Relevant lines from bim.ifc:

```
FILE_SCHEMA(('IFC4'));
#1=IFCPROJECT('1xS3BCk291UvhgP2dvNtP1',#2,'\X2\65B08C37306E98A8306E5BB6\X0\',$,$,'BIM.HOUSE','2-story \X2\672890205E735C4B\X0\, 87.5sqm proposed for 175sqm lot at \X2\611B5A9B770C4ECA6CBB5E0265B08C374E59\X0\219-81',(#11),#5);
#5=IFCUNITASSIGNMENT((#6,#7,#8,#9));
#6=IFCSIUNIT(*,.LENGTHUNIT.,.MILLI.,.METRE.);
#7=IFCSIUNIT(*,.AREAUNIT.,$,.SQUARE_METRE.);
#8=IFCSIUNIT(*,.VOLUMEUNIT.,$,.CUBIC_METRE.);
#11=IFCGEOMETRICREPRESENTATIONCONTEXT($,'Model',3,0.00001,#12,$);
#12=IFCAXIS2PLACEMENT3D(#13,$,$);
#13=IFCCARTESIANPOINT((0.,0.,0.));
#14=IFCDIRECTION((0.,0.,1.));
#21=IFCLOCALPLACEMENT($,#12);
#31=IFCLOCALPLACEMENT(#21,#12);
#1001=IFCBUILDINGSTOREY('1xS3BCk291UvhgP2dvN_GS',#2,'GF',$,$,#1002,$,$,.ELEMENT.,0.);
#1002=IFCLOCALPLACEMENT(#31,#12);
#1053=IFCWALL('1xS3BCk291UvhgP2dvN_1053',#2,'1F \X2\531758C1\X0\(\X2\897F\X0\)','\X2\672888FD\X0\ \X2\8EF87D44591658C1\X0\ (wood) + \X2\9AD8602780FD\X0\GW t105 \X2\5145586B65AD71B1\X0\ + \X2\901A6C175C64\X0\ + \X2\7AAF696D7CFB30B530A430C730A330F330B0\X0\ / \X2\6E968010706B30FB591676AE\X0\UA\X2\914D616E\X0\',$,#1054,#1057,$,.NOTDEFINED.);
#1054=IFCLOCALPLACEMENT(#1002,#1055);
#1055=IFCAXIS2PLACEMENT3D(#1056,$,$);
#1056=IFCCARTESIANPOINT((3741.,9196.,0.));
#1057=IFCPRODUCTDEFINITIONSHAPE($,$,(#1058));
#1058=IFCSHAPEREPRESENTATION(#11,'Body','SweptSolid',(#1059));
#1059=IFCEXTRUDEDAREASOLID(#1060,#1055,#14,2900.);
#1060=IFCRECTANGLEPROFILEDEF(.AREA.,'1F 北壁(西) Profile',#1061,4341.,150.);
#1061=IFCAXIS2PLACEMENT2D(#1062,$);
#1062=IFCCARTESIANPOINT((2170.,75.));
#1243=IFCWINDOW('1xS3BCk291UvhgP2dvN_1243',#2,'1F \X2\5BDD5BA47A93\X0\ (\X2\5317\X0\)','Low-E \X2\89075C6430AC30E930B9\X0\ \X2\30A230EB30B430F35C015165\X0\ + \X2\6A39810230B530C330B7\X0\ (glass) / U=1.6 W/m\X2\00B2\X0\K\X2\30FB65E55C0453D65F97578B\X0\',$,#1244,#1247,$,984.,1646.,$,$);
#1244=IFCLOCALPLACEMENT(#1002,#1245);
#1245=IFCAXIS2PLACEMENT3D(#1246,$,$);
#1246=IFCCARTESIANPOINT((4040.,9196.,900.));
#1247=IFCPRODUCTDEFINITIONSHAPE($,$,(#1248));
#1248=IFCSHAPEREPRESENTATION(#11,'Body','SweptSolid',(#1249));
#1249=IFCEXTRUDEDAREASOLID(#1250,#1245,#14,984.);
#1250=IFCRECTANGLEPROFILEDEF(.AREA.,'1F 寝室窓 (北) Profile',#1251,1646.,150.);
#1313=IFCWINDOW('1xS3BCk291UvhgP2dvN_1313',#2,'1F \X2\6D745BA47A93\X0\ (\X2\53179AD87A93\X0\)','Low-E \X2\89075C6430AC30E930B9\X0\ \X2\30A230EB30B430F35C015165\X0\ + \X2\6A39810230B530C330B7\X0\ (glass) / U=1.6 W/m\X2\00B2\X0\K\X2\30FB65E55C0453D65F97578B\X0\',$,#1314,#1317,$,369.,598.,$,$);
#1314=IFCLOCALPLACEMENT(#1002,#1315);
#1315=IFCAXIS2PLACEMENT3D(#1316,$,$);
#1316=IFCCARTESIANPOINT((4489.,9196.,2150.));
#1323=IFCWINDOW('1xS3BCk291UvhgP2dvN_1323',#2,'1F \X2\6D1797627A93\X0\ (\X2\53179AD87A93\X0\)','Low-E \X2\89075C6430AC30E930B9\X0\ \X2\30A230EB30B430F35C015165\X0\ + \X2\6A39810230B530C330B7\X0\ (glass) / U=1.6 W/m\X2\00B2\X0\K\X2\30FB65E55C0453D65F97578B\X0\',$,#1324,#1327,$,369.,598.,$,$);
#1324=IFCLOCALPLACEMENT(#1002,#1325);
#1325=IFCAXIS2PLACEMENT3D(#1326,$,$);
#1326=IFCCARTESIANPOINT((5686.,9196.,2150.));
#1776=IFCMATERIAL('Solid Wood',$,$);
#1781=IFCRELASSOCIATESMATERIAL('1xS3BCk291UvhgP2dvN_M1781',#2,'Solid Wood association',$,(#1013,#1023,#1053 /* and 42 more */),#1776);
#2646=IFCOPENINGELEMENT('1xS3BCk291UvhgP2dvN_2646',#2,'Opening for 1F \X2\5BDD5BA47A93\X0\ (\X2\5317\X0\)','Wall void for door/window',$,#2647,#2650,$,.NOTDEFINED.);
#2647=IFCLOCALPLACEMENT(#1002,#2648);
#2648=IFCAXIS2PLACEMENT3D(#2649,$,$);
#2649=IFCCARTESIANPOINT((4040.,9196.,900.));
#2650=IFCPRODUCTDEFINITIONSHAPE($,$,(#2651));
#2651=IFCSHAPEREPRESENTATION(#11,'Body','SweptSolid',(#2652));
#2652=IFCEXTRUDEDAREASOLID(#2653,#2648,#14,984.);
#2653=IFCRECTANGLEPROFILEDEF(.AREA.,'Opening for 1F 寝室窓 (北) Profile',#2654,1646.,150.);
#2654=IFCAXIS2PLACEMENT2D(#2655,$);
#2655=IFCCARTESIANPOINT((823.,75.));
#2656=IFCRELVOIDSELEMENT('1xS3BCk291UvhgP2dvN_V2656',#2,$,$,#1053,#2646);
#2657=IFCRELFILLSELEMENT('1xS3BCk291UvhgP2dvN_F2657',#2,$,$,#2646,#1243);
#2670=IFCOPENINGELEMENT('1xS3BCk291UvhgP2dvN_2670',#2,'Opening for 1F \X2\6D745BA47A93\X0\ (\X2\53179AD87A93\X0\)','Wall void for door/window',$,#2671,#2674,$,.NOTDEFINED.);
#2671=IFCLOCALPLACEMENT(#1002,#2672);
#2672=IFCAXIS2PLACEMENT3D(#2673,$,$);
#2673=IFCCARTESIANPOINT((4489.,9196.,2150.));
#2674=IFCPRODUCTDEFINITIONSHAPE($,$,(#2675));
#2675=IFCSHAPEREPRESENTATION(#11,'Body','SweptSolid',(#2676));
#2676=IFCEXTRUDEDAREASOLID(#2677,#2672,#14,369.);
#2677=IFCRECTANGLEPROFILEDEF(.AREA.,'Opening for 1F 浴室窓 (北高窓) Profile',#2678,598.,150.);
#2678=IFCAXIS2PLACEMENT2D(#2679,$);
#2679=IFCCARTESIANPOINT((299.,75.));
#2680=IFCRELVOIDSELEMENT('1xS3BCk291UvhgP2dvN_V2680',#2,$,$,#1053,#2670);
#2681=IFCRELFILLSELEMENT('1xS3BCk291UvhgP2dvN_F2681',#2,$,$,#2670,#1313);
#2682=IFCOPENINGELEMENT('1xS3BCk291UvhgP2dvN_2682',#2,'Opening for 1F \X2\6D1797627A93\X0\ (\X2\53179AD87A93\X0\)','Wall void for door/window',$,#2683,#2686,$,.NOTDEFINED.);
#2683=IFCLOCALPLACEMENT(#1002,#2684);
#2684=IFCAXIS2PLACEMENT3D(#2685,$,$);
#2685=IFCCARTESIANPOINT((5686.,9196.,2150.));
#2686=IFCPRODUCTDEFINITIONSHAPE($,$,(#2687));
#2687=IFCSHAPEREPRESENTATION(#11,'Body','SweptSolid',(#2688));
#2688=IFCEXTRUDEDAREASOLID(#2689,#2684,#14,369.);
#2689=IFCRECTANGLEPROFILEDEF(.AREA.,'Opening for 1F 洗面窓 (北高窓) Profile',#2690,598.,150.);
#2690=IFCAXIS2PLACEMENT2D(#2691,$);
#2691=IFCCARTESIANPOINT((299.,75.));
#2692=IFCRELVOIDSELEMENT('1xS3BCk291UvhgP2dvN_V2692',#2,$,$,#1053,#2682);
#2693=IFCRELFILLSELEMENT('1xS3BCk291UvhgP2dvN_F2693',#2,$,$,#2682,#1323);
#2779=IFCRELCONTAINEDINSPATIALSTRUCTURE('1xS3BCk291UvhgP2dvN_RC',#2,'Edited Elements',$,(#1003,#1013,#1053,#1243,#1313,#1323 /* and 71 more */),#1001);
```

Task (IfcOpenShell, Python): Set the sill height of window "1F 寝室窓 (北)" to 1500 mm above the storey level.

```python
import numpy as np
import ifcopenshell
import ifcopenshell.api.geometry
import ifcopenshell.geom
import ifcopenshell.util.element
import ifcopenshell.util.placement
import ifcopenshell.util.shape
import ifcopenshell.util.unit

model = ifcopenshell.open("bim.ifc")
unit_scale = ifcopenshell.util.unit.calculate_unit_scale(model)

window = model.by_id(1243)
opening = window.FillsVoids[0].RelatingOpeningElement
storey = ifcopenshell.util.element.get_container(window, ifc_class="IfcBuildingStorey")
level = ifcopenshell.util.placement.get_local_placement(storey.ObjectPlacement)[2, 3]

# The opening's origin need not be at the sill, so measure its lowest point.
shape = ifcopenshell.geom.create_shape(ifcopenshell.geom.settings(), opening)
bottom = ifcopenshell.util.shape.get_shape_bottom_elevation(shape, shape.geometry) / unit_scale
dz = level + 1.5 / unit_scale - bottom

shift = np.array([0.0, 0.0, dz])
# The window is not placed relative to its opening, so move both.
for product in (opening, window):
    matrix = ifcopenshell.util.placement.get_local_placement(product.ObjectPlacement)
    matrix[:3, 3] += shift
    ifcopenshell.api.geometry.edit_object_placement(model, product=product, matrix=matrix, is_si=False)

print(f"moved by {dz * unit_scale:+.3f} m")

model.write("bim_edited.ifc")
```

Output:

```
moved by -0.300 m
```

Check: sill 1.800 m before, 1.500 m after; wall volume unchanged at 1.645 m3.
